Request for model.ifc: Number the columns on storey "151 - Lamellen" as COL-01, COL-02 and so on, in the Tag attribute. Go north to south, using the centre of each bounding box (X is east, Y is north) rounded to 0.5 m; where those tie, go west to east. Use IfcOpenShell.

First a look at what the model holds.

```python
import ifcopenshell
import ifcopenshell.util.element
import ifcopenshell.util.placement

model = ifcopenshell.open("model.ifc")
print(model.schema)
storey = next(s for s in model.by_type("IfcBuildingStorey") if s.Name == "151 - Lamellen")
columns = [e for e in ifcopenshell.util.element.get_decomposition(storey) if e.is_a("IfcColumn")]
for e in sorted(columns, key=lambda e: e.id()):
    origin = ifcopenshell.util.placement.get_local_placement(e.ObjectPlacement)[:3, 3]
    print(e.id(), e.Tag, e.Name, origin.round(2) + 0.0, sep=" | ")
```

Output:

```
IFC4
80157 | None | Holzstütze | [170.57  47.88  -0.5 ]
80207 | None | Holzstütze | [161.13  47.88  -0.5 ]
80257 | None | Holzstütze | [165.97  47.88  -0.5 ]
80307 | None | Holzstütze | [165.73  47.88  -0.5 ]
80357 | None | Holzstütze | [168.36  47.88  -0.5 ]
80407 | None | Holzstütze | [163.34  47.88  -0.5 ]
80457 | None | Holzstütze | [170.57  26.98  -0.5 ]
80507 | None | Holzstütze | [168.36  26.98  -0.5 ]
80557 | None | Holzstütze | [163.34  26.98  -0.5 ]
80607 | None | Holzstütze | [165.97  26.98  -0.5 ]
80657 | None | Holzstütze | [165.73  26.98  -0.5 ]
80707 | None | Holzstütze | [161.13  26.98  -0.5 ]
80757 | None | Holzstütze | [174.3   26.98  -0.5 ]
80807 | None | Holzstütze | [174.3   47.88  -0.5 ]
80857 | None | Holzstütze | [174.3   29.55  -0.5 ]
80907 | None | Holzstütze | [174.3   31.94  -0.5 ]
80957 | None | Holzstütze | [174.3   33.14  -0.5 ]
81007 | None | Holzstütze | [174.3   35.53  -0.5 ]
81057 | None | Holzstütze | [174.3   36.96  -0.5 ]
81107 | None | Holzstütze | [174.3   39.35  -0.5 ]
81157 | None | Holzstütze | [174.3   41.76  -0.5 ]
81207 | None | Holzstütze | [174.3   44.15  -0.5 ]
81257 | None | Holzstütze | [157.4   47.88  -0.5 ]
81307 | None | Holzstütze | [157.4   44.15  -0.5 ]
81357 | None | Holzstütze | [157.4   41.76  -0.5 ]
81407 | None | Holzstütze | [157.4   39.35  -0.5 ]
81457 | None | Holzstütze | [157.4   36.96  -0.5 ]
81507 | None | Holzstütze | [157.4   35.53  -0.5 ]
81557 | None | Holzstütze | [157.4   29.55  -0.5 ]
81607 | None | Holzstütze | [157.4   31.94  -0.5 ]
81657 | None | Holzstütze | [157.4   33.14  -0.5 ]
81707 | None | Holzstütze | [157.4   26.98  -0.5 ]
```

```python
import ifcopenshell
import ifcopenshell.geom
import ifcopenshell.util.element
import ifcopenshell.util.shape

model = ifcopenshell.open("model.ifc")
settings = ifcopenshell.geom.settings()
settings.set("use-world-coords", True)


def centre(element):
    shape = ifcopenshell.geom.create_shape(settings, element)
    return ifcopenshell.util.shape.get_bbox_centroid(shape.geometry)


storey = next(s for s in model.by_type("IfcBuildingStorey") if s.Name == "151 - Lamellen")
columns = [e for e in ifcopenshell.util.element.get_decomposition(storey) if e.is_a("IfcColumn")]

# Insertion points can sit at a corner or the storey origin, so sort by the geometry (in metres).
centres = {e: centre(e) for e in columns}
columns.sort(key=lambda e: (-round(centres[e][1] / 0.5), centres[e][0]))

for i, e in enumerate(columns, start=1):
    number = f"COL-{i:02d}"
    e.Tag = number
    print(e.id(), number)

model.write("model_rev.ifc")
```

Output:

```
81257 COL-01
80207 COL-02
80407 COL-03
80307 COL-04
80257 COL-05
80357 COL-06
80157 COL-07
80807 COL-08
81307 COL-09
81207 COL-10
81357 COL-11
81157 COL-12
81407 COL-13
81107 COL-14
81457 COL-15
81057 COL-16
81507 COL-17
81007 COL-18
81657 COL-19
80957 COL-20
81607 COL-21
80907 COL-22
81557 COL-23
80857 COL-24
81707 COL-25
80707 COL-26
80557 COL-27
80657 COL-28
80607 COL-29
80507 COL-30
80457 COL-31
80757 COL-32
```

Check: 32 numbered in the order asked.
